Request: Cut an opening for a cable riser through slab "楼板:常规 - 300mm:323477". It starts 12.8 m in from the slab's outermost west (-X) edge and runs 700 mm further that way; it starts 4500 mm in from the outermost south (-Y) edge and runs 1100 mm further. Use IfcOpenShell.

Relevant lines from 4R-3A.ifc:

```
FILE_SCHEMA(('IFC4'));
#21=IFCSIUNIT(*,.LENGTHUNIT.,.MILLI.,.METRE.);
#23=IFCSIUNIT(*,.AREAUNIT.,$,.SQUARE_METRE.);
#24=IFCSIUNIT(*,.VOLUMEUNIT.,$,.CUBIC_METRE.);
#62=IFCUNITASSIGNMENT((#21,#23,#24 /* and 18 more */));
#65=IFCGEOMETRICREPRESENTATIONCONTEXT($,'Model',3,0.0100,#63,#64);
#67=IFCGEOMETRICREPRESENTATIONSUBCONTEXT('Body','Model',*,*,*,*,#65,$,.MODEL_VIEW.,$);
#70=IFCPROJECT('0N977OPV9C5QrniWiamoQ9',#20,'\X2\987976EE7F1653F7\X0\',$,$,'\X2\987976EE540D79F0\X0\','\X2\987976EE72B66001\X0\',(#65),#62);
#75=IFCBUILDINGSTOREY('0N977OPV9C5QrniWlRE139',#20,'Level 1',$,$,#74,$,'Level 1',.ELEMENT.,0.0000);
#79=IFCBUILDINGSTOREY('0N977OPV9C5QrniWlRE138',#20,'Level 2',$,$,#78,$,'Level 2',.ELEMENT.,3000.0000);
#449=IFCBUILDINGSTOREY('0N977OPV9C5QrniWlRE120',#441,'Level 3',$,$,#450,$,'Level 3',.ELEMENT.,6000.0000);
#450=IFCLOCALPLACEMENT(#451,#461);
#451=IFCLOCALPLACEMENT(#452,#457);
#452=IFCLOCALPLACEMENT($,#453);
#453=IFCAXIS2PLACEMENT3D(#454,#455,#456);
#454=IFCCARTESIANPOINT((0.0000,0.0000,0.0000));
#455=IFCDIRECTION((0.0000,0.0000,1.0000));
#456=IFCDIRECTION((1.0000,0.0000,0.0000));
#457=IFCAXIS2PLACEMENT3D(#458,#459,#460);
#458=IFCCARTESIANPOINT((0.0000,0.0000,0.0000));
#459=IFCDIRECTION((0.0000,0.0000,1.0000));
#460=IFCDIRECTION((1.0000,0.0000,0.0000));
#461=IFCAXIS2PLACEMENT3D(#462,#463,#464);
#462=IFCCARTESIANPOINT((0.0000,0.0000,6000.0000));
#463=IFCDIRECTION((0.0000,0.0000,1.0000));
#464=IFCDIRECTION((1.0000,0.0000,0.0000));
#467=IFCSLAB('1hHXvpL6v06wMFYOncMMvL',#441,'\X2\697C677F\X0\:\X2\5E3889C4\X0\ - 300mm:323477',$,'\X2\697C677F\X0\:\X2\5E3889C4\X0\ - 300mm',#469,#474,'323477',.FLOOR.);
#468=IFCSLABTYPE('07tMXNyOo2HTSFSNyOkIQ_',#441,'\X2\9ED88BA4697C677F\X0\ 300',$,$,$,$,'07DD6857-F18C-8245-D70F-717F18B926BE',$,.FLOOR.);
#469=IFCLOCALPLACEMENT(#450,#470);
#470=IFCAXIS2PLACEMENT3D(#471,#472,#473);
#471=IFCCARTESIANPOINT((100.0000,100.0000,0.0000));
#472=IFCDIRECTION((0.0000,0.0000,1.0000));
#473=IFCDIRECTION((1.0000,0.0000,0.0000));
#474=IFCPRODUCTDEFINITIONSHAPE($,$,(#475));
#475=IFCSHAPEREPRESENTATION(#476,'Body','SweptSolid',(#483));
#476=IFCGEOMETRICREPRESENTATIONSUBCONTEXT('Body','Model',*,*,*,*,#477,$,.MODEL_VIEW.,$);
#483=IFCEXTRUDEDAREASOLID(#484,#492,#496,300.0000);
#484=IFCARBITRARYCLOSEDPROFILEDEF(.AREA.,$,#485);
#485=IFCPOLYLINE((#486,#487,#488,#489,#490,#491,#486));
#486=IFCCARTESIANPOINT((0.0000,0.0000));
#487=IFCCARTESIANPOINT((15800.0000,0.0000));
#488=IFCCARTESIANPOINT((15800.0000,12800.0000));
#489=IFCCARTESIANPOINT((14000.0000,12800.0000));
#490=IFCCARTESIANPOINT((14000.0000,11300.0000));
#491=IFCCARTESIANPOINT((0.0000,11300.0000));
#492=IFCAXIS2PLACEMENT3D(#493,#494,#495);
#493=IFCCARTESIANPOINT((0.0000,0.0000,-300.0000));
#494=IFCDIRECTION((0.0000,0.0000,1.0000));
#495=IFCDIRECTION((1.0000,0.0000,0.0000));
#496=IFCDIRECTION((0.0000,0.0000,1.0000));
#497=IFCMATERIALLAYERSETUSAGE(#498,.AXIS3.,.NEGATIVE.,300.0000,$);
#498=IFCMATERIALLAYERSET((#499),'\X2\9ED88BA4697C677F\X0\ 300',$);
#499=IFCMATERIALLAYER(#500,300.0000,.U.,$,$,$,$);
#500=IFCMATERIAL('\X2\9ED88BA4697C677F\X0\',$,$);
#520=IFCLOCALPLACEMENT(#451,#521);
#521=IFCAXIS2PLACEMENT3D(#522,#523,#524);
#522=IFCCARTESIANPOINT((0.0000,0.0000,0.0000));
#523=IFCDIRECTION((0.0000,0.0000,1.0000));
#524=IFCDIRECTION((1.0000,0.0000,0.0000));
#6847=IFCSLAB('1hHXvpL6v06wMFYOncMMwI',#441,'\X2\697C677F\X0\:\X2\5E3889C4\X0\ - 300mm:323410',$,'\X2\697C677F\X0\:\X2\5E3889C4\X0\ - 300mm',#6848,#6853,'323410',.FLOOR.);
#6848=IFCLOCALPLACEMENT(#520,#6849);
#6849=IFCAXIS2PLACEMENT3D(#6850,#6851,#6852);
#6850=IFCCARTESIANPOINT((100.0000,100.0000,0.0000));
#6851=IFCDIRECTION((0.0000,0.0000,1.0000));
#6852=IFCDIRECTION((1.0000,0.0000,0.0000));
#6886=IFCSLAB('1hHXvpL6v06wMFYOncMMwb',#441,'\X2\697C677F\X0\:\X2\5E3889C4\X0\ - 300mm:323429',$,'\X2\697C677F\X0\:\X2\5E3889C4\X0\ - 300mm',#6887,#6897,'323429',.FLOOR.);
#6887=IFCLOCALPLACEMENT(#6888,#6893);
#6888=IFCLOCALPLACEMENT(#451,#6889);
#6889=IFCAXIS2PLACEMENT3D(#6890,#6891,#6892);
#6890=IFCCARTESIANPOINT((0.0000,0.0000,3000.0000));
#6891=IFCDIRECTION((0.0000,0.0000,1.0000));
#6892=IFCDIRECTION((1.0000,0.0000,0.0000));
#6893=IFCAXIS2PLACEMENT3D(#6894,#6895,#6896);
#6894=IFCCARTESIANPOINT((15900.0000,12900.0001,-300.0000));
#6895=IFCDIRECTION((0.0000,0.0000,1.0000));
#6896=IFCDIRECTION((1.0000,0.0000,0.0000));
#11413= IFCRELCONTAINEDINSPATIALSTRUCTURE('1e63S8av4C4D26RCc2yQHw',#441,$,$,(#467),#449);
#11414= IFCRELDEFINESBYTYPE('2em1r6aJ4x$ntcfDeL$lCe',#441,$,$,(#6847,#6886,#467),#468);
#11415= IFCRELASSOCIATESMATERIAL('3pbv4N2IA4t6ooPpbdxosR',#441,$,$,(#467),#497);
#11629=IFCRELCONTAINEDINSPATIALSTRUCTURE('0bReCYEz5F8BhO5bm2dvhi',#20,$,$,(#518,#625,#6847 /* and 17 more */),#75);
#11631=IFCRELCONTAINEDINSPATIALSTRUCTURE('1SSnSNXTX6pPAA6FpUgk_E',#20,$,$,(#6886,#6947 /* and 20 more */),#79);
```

```python
import numpy as np
import ifcopenshell
import ifcopenshell.api.feature
import ifcopenshell.api.geometry
import ifcopenshell.api.root
import ifcopenshell.geom
import ifcopenshell.util.placement
import ifcopenshell.util.representation
import ifcopenshell.util.shape
import ifcopenshell.util.unit

model = ifcopenshell.open("4R-3A.ifc")
unit_scale = ifcopenshell.util.unit.calculate_unit_scale(model)
settings = ifcopenshell.geom.settings()


def volume(element):
    """Net volume in cubic metres, openings subtracted."""
    shape = ifcopenshell.geom.create_shape(settings, element)
    return ifcopenshell.util.shape.get_volume(shape.geometry)


slab = model.by_id(467)
before = volume(slab)

# Extent in the slab's own axes, in metres. The edges named are its -X and -Y sides.
slab_shape = ifcopenshell.geom.create_shape(settings, slab)
vertices = ifcopenshell.util.shape.get_vertices(slab_shape.geometry)
x_min, y_min, bottom = vertices.min(axis=0)
top = vertices[:, 2].max()

opening = ifcopenshell.api.root.create_entity(model, ifc_class="IfcOpeningElement", name="Cable riser opening", predefined_type="OPENING")
context = ifcopenshell.util.representation.get_context(model, "Model", "Body", "MODEL_VIEW")
width, depth = 0.7, 1.1
outline = [(0.0, 0.0), (width, 0.0), (width, depth), (0.0, depth), (0.0, 0.0)]
# Overshoot both faces by 50 mm so the cut is clean.
shape = ifcopenshell.api.geometry.add_slab_representation(
    model, context=context, depth=top - bottom + 0.1, polyline=outline
)
ifcopenshell.api.geometry.assign_representation(model, product=opening, representation=shape)

matrix = ifcopenshell.util.placement.get_local_placement(slab.ObjectPlacement)
matrix[:, 3] = matrix @ np.append(np.array([x_min + 12.8, y_min + 4.5, bottom - 0.05]) / unit_scale, 1.0)
ifcopenshell.api.geometry.edit_object_placement(model, product=opening, matrix=matrix, is_si=False)
ifcopenshell.api.feature.add_feature(model, feature=opening, element=slab)

after = volume(slab)

print(f"slab volume {before:.3f} -> {after:.3f} m3")

model.write("4R-3A_edited.ifc")
```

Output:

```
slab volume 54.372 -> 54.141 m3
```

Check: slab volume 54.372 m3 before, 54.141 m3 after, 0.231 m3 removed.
